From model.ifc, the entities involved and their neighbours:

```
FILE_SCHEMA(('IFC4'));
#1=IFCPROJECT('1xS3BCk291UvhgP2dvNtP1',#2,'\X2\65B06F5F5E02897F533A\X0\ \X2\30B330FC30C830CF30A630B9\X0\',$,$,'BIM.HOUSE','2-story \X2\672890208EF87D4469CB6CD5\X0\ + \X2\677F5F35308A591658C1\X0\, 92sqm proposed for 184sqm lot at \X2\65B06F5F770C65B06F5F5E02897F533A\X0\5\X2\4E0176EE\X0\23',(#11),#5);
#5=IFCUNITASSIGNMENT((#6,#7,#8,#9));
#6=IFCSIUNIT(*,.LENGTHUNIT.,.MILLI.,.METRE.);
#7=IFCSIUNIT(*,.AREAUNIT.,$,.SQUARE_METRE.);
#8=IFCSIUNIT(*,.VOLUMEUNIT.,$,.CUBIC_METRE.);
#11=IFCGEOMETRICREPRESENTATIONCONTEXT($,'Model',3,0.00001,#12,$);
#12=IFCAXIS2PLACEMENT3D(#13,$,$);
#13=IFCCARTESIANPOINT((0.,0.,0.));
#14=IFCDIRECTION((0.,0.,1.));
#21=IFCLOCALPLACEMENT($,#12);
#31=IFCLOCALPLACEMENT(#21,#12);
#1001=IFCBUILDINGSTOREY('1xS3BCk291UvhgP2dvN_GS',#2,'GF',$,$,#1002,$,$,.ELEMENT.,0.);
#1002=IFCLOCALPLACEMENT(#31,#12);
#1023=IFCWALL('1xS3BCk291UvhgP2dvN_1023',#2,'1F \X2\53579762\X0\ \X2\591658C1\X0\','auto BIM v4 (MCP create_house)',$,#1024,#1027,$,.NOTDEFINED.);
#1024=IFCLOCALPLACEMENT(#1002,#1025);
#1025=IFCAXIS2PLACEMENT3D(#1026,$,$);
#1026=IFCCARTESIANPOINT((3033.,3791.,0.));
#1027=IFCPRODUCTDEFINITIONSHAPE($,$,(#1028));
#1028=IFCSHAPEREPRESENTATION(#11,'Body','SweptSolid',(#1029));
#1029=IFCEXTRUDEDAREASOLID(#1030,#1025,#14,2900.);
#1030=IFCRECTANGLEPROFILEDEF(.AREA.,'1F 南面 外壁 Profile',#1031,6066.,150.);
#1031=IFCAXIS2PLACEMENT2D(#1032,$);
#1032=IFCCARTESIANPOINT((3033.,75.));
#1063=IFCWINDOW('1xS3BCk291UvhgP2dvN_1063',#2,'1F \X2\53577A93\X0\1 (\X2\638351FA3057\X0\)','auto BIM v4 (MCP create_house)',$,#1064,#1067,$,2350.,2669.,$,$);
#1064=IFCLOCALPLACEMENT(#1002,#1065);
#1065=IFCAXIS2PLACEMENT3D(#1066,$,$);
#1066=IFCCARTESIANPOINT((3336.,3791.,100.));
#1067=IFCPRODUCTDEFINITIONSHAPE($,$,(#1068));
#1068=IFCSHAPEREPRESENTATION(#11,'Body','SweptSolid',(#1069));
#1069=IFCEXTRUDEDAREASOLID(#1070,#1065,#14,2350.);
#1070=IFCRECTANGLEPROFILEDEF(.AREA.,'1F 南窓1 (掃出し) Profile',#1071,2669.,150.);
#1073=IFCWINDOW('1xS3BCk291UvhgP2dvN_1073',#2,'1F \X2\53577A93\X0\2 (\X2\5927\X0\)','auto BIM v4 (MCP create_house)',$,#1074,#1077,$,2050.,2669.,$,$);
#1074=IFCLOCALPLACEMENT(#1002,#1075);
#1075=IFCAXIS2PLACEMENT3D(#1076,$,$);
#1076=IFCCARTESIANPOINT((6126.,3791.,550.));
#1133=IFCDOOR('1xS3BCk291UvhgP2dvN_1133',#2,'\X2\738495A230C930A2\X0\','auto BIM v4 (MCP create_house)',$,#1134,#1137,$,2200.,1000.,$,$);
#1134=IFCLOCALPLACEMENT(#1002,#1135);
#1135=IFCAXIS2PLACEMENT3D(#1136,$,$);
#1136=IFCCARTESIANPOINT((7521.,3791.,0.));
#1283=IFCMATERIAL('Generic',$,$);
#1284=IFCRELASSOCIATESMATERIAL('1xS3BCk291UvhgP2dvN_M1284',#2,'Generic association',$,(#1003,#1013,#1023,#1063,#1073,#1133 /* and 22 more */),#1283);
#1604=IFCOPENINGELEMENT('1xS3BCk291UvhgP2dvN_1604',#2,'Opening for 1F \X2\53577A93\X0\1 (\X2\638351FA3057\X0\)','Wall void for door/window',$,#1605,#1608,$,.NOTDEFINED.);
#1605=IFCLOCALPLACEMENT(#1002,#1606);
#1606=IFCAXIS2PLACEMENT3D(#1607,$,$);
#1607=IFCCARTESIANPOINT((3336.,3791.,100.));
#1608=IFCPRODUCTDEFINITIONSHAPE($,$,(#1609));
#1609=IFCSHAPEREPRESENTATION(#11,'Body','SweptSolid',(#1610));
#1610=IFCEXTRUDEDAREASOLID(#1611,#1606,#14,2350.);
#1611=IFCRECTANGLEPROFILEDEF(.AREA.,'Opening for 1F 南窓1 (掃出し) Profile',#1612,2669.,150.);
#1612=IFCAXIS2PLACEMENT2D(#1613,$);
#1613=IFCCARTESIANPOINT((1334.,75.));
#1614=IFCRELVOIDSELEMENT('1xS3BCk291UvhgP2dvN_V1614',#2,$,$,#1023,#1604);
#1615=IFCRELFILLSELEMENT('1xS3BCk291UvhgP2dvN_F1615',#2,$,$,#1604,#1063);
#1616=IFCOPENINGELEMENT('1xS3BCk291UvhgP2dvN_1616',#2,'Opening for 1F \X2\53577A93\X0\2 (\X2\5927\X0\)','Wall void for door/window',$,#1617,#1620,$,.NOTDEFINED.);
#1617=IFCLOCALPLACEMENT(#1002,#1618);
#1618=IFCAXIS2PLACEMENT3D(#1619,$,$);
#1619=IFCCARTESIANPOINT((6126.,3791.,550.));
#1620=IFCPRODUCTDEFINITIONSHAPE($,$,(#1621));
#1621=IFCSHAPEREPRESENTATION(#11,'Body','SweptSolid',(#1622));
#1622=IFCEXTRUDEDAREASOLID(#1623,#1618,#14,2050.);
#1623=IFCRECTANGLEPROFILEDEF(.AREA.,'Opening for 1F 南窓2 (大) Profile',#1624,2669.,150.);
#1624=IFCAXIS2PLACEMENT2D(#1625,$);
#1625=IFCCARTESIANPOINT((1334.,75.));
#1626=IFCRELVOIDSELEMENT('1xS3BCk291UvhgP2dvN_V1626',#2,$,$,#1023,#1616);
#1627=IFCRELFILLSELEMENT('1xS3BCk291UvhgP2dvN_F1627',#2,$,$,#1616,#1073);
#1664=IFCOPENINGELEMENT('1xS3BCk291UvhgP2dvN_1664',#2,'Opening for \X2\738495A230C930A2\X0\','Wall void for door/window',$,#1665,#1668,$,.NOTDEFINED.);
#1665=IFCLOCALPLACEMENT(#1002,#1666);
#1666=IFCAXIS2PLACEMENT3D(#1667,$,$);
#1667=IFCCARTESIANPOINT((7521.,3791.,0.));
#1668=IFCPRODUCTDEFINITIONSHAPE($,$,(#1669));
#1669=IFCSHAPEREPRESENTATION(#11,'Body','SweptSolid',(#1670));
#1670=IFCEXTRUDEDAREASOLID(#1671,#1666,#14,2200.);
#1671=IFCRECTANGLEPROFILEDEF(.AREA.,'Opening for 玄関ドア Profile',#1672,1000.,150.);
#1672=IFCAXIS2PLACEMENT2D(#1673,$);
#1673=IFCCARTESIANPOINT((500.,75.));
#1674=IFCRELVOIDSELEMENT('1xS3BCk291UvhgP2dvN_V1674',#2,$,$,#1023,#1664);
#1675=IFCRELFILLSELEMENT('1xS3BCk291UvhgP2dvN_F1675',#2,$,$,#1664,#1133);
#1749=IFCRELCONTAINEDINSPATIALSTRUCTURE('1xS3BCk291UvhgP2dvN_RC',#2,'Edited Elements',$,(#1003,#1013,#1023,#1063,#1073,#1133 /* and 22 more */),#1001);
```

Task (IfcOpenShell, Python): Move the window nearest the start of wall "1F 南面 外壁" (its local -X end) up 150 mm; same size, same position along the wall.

```python
import numpy as np
import ifcopenshell
import ifcopenshell.api.geometry
import ifcopenshell.util.placement
import ifcopenshell.util.unit

model = ifcopenshell.open("model.ifc")
unit_scale = ifcopenshell.util.unit.calculate_unit_scale(model)

window = model.by_id(1063)
opening = window.FillsVoids[0].RelatingOpeningElement
dz = 0.15 / unit_scale

shift = np.array([0.0, 0.0, dz])
# The window is not placed relative to its opening, so move both.
for product in (opening, window):
    matrix = ifcopenshell.util.placement.get_local_placement(product.ObjectPlacement)
    matrix[:3, 3] += shift
    ifcopenshell.api.geometry.edit_object_placement(model, product=product, matrix=matrix, is_si=False)

print(f"moved by {dz * unit_scale:+.3f} m")

model.write("model-out.ifc")
```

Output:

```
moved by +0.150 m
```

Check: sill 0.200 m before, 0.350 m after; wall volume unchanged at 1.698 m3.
